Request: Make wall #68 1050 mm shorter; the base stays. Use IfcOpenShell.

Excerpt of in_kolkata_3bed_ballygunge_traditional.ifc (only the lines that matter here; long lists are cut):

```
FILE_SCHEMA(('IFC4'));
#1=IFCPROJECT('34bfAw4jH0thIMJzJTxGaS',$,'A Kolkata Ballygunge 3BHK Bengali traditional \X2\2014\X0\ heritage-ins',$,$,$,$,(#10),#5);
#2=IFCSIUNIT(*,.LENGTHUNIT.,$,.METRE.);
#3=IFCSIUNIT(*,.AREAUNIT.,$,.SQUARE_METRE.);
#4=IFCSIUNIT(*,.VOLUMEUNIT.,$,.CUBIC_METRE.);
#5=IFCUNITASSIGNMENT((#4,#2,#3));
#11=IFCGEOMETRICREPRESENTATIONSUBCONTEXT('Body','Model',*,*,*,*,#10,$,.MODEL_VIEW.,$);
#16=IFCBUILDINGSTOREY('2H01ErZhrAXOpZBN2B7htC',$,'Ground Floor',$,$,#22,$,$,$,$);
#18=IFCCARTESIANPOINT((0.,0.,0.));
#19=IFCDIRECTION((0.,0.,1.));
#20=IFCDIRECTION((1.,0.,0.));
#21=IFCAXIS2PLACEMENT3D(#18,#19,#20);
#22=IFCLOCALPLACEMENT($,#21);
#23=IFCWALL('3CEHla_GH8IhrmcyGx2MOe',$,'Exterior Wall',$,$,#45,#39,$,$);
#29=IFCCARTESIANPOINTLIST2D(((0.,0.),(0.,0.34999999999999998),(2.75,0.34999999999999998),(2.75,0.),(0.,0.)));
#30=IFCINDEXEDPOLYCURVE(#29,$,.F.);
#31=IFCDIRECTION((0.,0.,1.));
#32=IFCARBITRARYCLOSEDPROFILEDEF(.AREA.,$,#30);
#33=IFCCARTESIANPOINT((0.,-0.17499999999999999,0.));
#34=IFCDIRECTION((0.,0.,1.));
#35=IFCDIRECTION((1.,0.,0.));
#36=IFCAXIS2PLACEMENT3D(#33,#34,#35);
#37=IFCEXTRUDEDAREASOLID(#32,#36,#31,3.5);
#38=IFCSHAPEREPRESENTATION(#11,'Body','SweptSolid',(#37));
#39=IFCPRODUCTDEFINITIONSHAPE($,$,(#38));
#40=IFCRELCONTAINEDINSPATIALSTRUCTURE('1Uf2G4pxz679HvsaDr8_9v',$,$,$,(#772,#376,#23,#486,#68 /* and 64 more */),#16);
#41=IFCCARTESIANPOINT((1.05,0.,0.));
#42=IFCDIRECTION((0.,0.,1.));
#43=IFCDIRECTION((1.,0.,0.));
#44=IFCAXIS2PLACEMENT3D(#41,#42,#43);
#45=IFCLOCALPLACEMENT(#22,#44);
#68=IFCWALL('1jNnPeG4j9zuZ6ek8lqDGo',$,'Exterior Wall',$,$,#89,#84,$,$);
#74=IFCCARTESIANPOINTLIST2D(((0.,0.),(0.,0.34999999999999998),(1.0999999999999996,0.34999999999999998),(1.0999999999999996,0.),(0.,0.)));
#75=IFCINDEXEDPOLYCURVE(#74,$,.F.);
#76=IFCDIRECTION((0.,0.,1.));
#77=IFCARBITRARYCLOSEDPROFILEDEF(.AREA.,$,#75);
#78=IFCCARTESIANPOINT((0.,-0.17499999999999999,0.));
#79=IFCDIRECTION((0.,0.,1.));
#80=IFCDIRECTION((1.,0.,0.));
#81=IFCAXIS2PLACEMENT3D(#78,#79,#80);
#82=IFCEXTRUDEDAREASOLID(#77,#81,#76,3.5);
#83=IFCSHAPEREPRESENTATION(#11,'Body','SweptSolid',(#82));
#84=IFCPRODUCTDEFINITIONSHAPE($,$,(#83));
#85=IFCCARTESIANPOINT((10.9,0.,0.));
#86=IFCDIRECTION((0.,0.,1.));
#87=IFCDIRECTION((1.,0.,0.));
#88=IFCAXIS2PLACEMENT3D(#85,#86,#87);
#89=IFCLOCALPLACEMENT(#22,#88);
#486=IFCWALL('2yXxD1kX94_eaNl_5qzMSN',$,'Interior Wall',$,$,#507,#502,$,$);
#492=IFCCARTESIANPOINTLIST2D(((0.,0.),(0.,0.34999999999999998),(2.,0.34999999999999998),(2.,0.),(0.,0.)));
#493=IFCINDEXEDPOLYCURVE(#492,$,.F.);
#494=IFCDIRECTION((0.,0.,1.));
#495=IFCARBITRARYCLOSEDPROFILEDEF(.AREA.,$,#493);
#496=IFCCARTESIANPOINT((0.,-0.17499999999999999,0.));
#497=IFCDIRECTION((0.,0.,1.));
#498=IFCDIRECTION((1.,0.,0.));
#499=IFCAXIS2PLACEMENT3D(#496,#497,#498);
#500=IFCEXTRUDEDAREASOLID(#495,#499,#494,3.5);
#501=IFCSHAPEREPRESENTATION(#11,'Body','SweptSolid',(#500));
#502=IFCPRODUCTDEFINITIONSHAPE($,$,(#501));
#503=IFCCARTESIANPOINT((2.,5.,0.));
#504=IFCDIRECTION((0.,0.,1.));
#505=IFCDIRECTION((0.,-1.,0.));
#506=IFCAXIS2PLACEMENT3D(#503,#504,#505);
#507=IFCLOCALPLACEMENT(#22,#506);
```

```python
import ifcopenshell
import ifcopenshell.geom
import ifcopenshell.util.representation
import ifcopenshell.util.shape

model = ifcopenshell.open("in_kolkata_3bed_ballygunge_traditional.ifc")
settings = ifcopenshell.geom.settings()


def volume(element):
    """Net volume in cubic metres, openings subtracted."""
    shape = ifcopenshell.geom.create_shape(settings, element)
    return ifcopenshell.util.shape.get_volume(shape.geometry)


wall = model.by_id(68)
before = volume(wall)

body = ifcopenshell.util.representation.get_representation(wall, "Model", "Body")
solid = body.Items[0]
old_height = solid.Depth
solid.Depth -= 1.05
after = volume(wall)

print(f"height {old_height:g} -> {solid.Depth:g}, volume {before:.3f} -> {after:.3f} m3")

model.write("in_kolkata_3bed_ballygunge_traditional-out.ifc")
```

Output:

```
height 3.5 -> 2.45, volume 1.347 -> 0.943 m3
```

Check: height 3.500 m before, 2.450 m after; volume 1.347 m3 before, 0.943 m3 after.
